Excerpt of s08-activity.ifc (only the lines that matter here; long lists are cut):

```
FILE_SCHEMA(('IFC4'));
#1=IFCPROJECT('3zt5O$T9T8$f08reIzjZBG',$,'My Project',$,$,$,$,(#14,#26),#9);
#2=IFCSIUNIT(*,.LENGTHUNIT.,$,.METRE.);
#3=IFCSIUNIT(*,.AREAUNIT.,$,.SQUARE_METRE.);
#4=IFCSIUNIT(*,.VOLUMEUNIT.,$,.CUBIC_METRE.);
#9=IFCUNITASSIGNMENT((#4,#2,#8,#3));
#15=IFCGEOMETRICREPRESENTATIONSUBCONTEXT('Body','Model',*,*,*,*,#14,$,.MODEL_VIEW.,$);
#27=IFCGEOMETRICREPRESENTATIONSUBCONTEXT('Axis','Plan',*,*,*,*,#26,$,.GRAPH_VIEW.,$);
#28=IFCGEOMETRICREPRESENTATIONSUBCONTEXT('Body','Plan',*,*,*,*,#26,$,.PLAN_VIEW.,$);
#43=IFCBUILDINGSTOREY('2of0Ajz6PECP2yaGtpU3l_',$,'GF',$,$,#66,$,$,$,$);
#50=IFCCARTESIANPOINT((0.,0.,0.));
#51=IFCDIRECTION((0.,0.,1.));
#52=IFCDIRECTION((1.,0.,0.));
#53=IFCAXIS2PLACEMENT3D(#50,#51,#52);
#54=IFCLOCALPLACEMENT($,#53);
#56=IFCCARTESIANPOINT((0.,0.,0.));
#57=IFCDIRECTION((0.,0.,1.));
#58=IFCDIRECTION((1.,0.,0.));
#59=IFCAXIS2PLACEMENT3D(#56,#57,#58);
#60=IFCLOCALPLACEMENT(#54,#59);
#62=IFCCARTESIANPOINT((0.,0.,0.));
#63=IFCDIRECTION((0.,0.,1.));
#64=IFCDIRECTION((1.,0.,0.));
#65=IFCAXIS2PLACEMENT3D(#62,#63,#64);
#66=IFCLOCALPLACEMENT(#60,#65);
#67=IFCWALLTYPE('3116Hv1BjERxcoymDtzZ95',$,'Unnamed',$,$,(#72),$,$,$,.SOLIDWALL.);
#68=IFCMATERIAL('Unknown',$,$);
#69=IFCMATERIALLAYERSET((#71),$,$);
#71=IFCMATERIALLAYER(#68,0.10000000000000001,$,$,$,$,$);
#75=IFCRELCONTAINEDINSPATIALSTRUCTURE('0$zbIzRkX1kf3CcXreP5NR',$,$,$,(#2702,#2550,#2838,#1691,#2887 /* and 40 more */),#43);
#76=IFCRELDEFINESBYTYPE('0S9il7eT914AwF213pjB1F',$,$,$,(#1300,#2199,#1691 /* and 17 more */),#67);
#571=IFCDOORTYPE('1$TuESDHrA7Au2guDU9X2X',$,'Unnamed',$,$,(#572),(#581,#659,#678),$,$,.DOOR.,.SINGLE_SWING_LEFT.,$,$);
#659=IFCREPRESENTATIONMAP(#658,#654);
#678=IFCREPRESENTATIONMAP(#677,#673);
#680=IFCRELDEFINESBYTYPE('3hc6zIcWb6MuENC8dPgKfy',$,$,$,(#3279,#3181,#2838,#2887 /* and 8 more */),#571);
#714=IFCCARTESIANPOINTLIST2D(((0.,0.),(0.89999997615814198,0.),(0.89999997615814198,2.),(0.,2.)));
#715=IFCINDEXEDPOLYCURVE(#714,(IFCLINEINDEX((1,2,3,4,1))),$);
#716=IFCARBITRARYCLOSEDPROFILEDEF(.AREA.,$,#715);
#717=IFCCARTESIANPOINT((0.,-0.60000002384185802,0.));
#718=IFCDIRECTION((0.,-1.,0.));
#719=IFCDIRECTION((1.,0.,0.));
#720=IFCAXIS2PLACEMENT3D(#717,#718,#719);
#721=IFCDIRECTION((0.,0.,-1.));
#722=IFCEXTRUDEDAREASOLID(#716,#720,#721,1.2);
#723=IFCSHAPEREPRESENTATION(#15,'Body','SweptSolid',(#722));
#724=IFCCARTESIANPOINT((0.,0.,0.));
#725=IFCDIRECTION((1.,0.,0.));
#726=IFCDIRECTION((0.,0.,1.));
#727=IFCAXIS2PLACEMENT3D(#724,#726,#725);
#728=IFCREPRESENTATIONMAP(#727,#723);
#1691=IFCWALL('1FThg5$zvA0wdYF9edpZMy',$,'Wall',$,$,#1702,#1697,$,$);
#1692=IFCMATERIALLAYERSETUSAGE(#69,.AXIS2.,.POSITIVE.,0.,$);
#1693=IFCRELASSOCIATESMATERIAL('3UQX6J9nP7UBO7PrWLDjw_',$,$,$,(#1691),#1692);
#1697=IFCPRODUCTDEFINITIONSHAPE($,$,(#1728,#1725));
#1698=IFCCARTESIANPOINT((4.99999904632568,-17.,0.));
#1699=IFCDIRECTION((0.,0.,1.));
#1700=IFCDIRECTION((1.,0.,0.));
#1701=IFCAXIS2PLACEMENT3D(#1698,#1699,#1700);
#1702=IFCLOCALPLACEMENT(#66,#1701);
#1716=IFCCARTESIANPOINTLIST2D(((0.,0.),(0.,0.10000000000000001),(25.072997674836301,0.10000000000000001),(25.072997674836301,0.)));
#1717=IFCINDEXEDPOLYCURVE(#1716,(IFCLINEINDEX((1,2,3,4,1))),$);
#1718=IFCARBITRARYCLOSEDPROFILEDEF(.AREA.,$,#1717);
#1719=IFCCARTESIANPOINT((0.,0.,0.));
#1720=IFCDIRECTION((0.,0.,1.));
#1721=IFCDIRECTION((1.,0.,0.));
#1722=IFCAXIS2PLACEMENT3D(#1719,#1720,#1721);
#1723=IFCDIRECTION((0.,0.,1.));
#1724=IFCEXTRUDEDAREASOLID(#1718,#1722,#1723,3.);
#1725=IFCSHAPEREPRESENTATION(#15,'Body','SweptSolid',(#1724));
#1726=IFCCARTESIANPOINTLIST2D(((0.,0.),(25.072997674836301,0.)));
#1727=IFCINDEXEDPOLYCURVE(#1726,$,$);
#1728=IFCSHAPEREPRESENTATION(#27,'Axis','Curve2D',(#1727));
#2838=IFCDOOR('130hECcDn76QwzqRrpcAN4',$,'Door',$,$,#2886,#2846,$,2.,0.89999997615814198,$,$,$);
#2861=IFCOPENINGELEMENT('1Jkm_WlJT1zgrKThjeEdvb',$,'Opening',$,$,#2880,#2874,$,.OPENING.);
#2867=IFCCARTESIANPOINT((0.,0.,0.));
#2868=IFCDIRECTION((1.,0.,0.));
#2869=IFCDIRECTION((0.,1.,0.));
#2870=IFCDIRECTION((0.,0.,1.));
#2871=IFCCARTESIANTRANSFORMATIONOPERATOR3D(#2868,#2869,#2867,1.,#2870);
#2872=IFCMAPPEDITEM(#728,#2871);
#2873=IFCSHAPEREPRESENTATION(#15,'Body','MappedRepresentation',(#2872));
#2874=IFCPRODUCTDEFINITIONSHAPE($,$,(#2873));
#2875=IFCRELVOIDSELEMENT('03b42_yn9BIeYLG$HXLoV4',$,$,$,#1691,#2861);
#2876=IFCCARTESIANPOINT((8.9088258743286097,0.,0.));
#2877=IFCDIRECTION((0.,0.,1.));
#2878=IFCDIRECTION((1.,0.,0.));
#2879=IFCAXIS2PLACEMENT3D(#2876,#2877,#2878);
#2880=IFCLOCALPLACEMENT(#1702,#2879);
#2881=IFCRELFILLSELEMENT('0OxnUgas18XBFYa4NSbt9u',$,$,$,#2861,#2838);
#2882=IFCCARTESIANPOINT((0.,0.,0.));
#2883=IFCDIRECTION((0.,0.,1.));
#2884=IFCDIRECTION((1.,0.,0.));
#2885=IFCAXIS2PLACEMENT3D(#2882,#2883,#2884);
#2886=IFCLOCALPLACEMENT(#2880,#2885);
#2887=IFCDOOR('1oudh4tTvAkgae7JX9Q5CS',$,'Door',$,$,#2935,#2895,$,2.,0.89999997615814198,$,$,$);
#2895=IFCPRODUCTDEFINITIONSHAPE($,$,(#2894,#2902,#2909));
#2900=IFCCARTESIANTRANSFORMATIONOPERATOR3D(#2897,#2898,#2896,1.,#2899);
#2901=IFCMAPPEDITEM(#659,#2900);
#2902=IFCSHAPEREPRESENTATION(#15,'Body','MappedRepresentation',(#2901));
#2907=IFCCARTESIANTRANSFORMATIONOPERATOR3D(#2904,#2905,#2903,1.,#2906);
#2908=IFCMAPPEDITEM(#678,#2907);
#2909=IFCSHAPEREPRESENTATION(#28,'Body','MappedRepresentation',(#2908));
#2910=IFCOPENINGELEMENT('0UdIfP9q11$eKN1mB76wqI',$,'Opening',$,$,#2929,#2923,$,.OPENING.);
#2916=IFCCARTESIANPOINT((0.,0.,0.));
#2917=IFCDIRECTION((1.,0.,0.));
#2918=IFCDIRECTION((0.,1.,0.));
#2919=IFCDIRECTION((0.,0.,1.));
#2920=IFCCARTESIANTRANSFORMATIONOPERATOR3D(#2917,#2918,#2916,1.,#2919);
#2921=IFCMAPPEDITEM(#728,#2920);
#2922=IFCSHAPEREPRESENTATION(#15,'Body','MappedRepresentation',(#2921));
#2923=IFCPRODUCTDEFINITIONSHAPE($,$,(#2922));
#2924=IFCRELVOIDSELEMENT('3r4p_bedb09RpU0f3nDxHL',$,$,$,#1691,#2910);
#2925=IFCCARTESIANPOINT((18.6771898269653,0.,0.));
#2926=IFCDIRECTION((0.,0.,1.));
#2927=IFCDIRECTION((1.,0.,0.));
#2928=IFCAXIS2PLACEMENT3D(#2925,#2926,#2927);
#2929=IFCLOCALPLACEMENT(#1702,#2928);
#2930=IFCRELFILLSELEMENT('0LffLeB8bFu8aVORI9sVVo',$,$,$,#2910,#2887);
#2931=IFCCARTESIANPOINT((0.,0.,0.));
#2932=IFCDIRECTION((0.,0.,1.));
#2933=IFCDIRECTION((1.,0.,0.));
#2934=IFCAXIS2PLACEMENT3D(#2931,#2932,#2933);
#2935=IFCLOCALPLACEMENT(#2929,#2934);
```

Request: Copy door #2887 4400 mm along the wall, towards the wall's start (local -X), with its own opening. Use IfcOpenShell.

```python
import ifcopenshell
import ifcopenshell.api.feature
import ifcopenshell.api.geometry
import ifcopenshell.api.root
import ifcopenshell.geom
import ifcopenshell.util.element
import ifcopenshell.util.placement
import ifcopenshell.util.shape
import ifcopenshell.util.unit

model = ifcopenshell.open("s08-activity.ifc")
unit_scale = ifcopenshell.util.unit.calculate_unit_scale(model)
settings = ifcopenshell.geom.settings()


def volume(element):
    """Net volume in cubic metres, openings subtracted."""
    shape = ifcopenshell.geom.create_shape(settings, element)
    return ifcopenshell.util.shape.get_volume(shape.geometry)


door = model.by_id(2887)
opening = door.FillsVoids[0].RelatingOpeningElement
wall = opening.VoidsElements[0].RelatingBuildingElement
before = volume(wall)
shift = ifcopenshell.util.placement.get_local_placement(wall.ObjectPlacement)[:3, 0] * -4.4 / unit_scale

# copy_class copies the void relationship, type, container and properties, but no geometry.
new_opening = ifcopenshell.api.root.copy_class(model, product=opening)
new_opening.Representation = ifcopenshell.util.element.copy_deep(
    model, opening.Representation, exclude=["IfcGeometricRepresentationContext", "IfcRepresentationMap"]
)
new_door = ifcopenshell.api.root.copy_class(model, product=door)
new_door.Representation = ifcopenshell.util.element.copy_deep(
    model, door.Representation, exclude=["IfcGeometricRepresentationContext", "IfcRepresentationMap"]
)
ifcopenshell.api.feature.add_filling(model, opening=new_opening, element=new_door)

for old, new in ((opening, new_opening), (door, new_door)):
    matrix = ifcopenshell.util.placement.get_local_placement(old.ObjectPlacement)
    matrix[:3, 3] += shift
    ifcopenshell.api.geometry.edit_object_placement(model, product=new, matrix=matrix, is_si=False)

after = volume(wall)

print(f"wall volume {before:.3f} -> {after:.3f} m3")

model.write("s08-activity_rev.ifc")
```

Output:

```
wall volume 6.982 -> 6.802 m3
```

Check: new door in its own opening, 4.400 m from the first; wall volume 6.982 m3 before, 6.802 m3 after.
